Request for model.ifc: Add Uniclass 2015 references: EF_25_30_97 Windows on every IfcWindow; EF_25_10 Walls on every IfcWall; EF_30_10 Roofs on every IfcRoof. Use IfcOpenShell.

First a look at what the model holds.

```python
import ifcopenshell

model = ifcopenshell.open("model.ifc")
print(model.schema)
print("classifications:", [c.Name for c in model.by_type("IfcClassification")])
for ifc_class in ("IfcDoor", "IfcRoof", "IfcStair", "IfcWall", "IfcWindow"):
    print(ifc_class, len(model.by_type(ifc_class)))
```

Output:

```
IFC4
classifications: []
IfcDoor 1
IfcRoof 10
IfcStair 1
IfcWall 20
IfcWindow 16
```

```python
import ifcopenshell
import ifcopenshell.api.classification

model = ifcopenshell.open("model.ifc")

system = ifcopenshell.api.classification.add_classification(model, classification="Uniclass 2015")

codes = {
    "IfcWindow": ("EF_25_30_97", "Windows"),
    "IfcWall": ("EF_25_10", "Walls"),
    "IfcRoof": ("EF_30_10", "Roofs"),
}
for ifc_class, (code, name) in codes.items():
    products = model.by_type(ifc_class)
    ifcopenshell.api.classification.add_reference(
        model, products=products, classification=system, identification=code, name=name
    )
    print(code, len(products))

model.write("model_v2.ifc")
```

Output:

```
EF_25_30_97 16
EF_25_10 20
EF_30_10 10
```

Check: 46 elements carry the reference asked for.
